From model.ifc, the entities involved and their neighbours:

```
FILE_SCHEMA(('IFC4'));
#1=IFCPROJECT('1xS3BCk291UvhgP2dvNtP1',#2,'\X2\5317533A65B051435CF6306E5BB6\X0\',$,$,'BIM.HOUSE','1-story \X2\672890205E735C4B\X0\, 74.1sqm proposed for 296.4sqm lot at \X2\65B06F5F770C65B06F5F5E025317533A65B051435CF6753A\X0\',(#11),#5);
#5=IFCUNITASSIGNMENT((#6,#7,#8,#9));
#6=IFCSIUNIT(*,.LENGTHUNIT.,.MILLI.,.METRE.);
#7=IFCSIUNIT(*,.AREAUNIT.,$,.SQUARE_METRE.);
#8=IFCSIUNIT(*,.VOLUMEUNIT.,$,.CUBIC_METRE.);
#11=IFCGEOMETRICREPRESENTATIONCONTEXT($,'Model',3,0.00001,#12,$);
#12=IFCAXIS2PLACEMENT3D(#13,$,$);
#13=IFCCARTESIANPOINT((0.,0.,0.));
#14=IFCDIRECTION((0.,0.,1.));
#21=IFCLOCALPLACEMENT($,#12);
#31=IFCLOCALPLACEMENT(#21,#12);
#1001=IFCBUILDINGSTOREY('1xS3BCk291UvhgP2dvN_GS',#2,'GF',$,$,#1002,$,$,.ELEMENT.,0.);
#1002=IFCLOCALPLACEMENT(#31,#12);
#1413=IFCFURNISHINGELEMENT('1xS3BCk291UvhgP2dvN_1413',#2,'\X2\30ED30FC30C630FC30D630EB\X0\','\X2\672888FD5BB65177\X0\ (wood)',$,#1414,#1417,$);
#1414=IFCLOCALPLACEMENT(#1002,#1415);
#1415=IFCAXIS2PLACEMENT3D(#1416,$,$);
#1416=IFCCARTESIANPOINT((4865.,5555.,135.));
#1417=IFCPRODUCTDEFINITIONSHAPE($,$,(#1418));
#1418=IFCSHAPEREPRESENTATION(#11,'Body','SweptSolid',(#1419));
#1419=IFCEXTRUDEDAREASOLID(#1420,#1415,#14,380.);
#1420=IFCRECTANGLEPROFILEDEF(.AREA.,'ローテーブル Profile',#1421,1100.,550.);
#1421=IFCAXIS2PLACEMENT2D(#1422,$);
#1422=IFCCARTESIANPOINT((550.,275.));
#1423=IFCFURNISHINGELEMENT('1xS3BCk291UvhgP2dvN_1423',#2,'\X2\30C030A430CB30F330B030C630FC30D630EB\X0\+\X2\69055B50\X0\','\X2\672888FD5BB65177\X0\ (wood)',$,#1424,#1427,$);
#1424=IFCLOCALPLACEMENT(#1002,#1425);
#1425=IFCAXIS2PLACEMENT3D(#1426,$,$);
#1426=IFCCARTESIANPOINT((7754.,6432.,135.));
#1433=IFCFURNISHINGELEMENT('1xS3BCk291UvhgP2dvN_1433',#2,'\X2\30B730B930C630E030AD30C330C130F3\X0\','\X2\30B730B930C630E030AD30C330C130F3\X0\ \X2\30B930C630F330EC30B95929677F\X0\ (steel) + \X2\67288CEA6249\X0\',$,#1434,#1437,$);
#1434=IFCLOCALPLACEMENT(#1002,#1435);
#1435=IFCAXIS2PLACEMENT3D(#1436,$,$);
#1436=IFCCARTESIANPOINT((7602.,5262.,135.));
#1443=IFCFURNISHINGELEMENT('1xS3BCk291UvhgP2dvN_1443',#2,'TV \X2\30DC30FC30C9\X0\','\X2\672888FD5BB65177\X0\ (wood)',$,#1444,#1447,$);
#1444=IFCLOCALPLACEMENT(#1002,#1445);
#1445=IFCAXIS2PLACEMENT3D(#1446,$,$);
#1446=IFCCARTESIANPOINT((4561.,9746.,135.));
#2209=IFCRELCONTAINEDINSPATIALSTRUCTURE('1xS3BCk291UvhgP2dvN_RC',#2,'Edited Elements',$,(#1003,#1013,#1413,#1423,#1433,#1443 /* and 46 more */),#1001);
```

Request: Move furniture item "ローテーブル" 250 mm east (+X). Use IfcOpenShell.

```python
import ifcopenshell
import ifcopenshell.api.geometry
import ifcopenshell.util.placement

model = ifcopenshell.open("model.ifc")

item = model.by_guid("1xS3BCk291UvhgP2dvN_1413")
matrix = ifcopenshell.util.placement.get_local_placement(item.ObjectPlacement)
matrix[0, 3] += 250.0
ifcopenshell.api.geometry.edit_object_placement(model, product=item, matrix=matrix, is_si=False)

print(ifcopenshell.util.placement.get_local_placement(item.ObjectPlacement).round(3) + 0.0)

model.write("model_rev.ifc")
```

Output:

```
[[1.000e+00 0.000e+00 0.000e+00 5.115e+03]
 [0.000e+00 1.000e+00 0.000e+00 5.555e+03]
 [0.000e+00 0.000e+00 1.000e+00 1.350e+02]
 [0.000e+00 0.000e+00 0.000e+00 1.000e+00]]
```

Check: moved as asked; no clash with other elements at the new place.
